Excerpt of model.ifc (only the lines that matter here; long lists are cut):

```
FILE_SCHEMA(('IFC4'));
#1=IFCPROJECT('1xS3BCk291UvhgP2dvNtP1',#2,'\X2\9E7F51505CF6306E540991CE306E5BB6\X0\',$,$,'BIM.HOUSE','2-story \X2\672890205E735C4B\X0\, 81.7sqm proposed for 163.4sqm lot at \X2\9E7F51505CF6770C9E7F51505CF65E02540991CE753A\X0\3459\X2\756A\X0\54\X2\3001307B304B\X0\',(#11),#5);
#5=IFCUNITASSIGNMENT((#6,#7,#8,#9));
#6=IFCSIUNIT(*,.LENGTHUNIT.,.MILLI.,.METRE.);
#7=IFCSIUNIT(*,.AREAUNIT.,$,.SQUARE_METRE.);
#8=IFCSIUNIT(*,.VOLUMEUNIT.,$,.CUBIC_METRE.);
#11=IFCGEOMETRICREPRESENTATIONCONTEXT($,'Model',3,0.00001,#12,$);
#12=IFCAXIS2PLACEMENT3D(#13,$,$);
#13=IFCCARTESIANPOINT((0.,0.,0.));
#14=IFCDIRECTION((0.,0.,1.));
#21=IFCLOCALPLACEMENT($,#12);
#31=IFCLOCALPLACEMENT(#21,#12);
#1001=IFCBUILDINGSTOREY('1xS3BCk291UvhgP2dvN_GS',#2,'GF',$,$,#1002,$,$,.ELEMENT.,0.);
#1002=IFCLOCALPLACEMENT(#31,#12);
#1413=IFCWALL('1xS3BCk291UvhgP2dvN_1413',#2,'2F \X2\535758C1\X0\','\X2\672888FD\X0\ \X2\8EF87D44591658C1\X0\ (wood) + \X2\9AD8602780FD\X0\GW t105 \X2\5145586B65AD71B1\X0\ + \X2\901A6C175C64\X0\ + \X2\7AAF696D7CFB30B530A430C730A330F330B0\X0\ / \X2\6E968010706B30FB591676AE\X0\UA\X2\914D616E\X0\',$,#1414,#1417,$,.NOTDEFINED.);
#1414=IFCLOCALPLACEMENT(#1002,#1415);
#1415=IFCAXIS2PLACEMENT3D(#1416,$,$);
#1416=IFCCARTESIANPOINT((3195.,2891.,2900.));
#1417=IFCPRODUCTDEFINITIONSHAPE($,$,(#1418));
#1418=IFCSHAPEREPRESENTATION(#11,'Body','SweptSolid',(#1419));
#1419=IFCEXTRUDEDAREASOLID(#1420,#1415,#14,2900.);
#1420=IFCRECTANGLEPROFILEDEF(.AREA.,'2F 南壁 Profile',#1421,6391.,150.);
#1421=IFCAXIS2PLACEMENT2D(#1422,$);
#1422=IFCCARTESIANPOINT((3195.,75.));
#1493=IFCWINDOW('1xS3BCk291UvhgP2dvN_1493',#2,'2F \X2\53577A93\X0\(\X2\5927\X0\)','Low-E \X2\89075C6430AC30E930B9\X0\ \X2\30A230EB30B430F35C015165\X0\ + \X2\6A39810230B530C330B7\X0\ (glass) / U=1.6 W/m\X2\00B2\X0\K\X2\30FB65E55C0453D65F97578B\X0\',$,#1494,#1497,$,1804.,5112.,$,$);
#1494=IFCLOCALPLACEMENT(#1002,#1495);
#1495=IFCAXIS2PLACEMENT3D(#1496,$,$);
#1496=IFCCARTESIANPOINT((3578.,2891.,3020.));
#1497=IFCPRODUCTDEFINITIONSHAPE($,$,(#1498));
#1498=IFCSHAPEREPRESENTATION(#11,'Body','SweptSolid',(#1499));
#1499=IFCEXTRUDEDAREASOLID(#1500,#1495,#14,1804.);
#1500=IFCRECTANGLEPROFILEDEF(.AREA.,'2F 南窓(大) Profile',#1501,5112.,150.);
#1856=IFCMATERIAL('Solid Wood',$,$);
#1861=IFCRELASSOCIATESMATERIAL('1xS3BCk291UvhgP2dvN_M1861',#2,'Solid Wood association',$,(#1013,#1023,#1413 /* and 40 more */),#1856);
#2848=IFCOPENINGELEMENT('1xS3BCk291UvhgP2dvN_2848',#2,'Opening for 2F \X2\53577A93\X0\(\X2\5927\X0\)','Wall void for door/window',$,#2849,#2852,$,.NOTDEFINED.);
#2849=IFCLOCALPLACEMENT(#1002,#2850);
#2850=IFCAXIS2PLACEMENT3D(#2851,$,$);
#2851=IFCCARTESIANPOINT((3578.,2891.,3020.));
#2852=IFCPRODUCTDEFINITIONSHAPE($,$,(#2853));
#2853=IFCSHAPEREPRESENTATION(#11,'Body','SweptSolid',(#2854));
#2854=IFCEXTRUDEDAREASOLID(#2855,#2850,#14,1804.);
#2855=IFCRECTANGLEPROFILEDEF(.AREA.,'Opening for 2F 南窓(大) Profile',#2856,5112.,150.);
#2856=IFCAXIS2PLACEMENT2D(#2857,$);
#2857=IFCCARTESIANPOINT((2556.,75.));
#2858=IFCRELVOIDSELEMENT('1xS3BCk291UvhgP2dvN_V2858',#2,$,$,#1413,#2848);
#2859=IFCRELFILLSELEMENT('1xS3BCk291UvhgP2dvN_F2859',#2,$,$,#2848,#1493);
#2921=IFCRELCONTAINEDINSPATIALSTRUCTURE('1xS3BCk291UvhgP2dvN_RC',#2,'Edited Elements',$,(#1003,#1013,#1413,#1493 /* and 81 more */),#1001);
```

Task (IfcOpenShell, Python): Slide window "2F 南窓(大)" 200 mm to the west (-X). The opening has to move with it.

```python
import ifcopenshell
import ifcopenshell.api.geometry
import ifcopenshell.util.placement
import ifcopenshell.util.unit

model = ifcopenshell.open("model.ifc")
unit_scale = ifcopenshell.util.unit.calculate_unit_scale(model)

window = model.by_guid("1xS3BCk291UvhgP2dvN_1493")
opening = window.FillsVoids[0].RelatingOpeningElement
wall = opening.VoidsElements[0].RelatingBuildingElement

wall_matrix = ifcopenshell.util.placement.get_local_placement(wall.ObjectPlacement)
shift = wall_matrix[:3, 0] * -0.2 / unit_scale
before = ifcopenshell.util.placement.get_local_placement(window.ObjectPlacement)[:3, 3].copy()

# The window is not placed relative to its opening, so move both.
for product in (opening, window):
    matrix = ifcopenshell.util.placement.get_local_placement(product.ObjectPlacement)
    matrix[:3, 3] += shift
    ifcopenshell.api.geometry.edit_object_placement(model, product=product, matrix=matrix, is_si=False)

after = ifcopenshell.util.placement.get_local_placement(window.ObjectPlacement)[:3, 3]
print("window moved by", (after - before).round(3) + 0.0)

model.write("model_updated.ifc")
```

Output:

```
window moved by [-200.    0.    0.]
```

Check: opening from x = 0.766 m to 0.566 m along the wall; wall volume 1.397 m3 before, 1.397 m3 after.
